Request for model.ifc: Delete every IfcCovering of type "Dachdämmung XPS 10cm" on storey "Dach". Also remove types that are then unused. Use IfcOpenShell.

First a look at what the model holds.

```python
import ifcopenshell
import ifcopenshell.util.element

model = ifcopenshell.open("model.ifc")
print(model.schema)
storey = next(s for s in model.by_type("IfcBuildingStorey") if s.Name == "Dach")
coverings = [e for e in ifcopenshell.util.element.get_decomposition(storey) if e.is_a("IfcCovering")]
seen = {}
for e in coverings:
    element_type = ifcopenshell.util.element.get_type(e)
    name = element_type.Name if element_type not in (None, e) else None
    seen[name] = seen.get(name, 0) + 1
for name, count in sorted(seen.items(), key=str):
    print(count, "x", name)
```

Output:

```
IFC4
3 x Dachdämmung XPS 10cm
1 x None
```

```python
import ifcopenshell
import ifcopenshell.api.root
import ifcopenshell.util.element

model = ifcopenshell.open("model.ifc")

storey = next(s for s in model.by_type("IfcBuildingStorey") if s.Name == "Dach")
coverings = [e for e in ifcopenshell.util.element.get_decomposition(storey) if e.is_a("IfcCovering")]
targets = [e for e in coverings if (t := ifcopenshell.util.element.get_type(e)) not in (None, e) and t.Name == "Dachdämmung XPS 10cm"]
types = {ifcopenshell.util.element.get_type(e) for e in targets} - {None, *targets}

for e in targets:
    ifcopenshell.api.root.remove_product(model, product=e)
print(len(targets), "removed")

unused = [t for t in types if not ifcopenshell.util.element.get_types(t)]
for t in unused:
    ifcopenshell.api.root.remove_product(model, product=t)
print(len(unused), "unused types removed")

model.write("model_updated.ifc")
```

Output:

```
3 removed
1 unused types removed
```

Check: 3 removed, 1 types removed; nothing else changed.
